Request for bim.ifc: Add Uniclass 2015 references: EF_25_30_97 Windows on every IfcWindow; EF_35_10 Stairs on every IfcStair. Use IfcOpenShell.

First a look at what the model holds.

```python
import ifcopenshell

model = ifcopenshell.open("bim.ifc")
print(model.schema)
print("classifications:", [c.Name for c in model.by_type("IfcClassification")])
for ifc_class in ("IfcDoor", "IfcRoof", "IfcStair", "IfcWall", "IfcWindow"):
    print(ifc_class, len(model.by_type(ifc_class)))
```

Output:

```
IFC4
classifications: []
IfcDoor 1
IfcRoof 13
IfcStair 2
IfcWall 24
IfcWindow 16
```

```python
import ifcopenshell
import ifcopenshell.api.classification

model = ifcopenshell.open("bim.ifc")

system = ifcopenshell.api.classification.add_classification(model, classification="Uniclass 2015")

codes = {
    "IfcWindow": ("EF_25_30_97", "Windows"),
    "IfcStair": ("EF_35_10", "Stairs"),
}
for ifc_class, (code, name) in codes.items():
    products = model.by_type(ifc_class)
    ifcopenshell.api.classification.add_reference(
        model, products=products, classification=system, identification=code, name=name
    )
    print(code, len(products))

model.write("bim_v2.ifc")
```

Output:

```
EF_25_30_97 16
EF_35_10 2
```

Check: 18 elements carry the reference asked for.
